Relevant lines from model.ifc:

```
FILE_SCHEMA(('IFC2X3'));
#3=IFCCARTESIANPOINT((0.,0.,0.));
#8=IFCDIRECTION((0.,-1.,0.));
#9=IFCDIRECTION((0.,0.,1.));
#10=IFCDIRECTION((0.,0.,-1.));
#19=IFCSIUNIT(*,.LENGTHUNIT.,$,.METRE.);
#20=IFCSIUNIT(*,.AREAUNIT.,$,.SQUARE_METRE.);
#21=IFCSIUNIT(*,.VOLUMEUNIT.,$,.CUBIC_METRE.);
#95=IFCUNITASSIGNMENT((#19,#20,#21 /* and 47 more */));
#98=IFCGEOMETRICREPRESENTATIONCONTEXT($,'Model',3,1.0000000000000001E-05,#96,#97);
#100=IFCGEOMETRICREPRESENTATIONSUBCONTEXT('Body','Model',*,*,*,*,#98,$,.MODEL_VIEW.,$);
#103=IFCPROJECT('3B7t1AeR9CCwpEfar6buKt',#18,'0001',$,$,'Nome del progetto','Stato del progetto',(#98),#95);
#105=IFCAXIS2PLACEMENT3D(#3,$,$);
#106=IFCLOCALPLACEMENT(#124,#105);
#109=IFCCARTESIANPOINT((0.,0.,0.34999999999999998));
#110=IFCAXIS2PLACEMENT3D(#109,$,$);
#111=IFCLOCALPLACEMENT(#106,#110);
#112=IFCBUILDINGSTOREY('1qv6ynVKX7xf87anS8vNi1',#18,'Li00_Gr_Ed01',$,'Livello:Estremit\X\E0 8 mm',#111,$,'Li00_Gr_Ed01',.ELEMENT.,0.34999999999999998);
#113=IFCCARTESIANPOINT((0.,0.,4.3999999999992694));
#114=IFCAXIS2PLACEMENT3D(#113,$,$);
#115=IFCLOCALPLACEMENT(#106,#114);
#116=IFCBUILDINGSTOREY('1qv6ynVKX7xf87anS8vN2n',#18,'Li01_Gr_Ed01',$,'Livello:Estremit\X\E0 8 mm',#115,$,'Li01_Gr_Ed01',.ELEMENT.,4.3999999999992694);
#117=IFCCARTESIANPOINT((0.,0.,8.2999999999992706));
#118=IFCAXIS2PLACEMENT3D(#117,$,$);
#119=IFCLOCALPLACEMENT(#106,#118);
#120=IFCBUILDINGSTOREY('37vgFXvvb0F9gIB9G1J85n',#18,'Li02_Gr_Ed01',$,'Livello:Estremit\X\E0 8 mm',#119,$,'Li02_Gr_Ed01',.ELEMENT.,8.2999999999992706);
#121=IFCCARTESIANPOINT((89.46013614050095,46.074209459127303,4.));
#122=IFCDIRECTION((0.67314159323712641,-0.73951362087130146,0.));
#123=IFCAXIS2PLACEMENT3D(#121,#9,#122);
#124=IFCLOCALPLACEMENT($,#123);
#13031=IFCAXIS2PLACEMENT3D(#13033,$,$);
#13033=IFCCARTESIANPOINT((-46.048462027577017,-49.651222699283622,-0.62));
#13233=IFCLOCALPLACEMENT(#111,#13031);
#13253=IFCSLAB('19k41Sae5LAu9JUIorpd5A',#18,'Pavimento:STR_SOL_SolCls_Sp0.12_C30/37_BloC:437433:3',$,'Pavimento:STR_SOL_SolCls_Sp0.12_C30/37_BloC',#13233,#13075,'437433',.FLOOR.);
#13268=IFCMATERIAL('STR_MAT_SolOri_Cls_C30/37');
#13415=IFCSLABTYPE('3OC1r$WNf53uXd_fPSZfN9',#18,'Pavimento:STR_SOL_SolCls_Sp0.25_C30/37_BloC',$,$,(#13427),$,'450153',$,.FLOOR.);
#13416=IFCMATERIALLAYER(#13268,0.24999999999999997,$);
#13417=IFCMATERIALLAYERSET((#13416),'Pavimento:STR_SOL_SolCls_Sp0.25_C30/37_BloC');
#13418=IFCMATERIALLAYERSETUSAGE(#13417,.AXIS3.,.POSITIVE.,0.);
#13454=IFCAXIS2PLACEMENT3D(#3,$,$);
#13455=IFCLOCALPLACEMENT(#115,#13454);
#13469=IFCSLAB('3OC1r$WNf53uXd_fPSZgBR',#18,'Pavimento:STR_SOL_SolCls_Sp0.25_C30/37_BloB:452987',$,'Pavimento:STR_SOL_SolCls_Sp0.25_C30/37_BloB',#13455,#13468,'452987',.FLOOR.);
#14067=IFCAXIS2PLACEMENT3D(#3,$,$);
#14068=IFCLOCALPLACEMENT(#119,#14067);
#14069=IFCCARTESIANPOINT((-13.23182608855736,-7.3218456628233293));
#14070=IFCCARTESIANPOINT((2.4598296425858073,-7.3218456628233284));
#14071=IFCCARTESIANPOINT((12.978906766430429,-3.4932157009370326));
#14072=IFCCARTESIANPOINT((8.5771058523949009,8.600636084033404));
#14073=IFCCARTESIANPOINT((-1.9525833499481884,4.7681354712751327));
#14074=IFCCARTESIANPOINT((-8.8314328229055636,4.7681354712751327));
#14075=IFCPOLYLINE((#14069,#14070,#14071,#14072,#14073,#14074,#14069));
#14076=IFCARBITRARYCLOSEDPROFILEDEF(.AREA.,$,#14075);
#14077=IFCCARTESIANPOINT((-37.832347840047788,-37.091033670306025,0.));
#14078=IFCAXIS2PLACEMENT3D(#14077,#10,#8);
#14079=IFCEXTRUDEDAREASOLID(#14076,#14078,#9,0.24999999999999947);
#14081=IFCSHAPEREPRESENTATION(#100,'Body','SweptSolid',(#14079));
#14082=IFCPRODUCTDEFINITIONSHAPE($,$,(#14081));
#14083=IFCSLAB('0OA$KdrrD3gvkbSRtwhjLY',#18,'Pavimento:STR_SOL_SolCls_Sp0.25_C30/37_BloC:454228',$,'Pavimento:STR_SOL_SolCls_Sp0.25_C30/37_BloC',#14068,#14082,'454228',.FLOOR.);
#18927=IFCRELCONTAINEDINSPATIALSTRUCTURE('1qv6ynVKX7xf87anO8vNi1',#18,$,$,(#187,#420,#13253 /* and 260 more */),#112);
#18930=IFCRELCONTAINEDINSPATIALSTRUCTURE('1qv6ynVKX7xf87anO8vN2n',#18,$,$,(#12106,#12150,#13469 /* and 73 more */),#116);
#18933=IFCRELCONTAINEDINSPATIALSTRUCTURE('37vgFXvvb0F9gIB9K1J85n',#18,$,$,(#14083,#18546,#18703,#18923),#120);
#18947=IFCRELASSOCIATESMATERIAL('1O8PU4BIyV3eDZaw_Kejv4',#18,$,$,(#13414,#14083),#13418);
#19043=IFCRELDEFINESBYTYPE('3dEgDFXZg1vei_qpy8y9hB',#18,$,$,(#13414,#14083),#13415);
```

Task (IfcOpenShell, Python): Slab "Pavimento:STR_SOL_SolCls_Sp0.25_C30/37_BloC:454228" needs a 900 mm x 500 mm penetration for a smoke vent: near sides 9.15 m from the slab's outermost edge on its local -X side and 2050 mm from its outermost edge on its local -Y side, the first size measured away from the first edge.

```python
import numpy as np
import ifcopenshell
import ifcopenshell.api.feature
import ifcopenshell.api.geometry
import ifcopenshell.api.root
import ifcopenshell.geom
import ifcopenshell.util.placement
import ifcopenshell.util.representation
import ifcopenshell.util.shape
import ifcopenshell.util.unit

model = ifcopenshell.open("model.ifc")
unit_scale = ifcopenshell.util.unit.calculate_unit_scale(model)
settings = ifcopenshell.geom.settings()


def volume(element):
    """Net volume in cubic metres, openings subtracted."""
    shape = ifcopenshell.geom.create_shape(settings, element)
    return ifcopenshell.util.shape.get_volume(shape.geometry)


slab = model.by_id(14083)
before = volume(slab)

# Extent in the slab's own axes, in metres. The edges named are its -X and -Y sides.
slab_shape = ifcopenshell.geom.create_shape(settings, slab)
vertices = ifcopenshell.util.shape.get_vertices(slab_shape.geometry)
x_min, y_min, bottom = vertices.min(axis=0)
top = vertices[:, 2].max()

opening = ifcopenshell.api.root.create_entity(model, ifc_class="IfcOpeningElement", name="Smoke vent opening")
context = ifcopenshell.util.representation.get_context(model, "Model", "Body", "MODEL_VIEW")
width, depth = 0.9, 0.5
outline = [(0.0, 0.0), (width, 0.0), (width, depth), (0.0, depth), (0.0, 0.0)]
# Overshoot both faces by 50 mm so the cut is clean.
shape = ifcopenshell.api.geometry.add_slab_representation(
    model, context=context, depth=top - bottom + 0.1, polyline=outline
)
ifcopenshell.api.geometry.assign_representation(model, product=opening, representation=shape)

matrix = ifcopenshell.util.placement.get_local_placement(slab.ObjectPlacement)
matrix[:, 3] = matrix @ np.append(np.array([x_min + 9.15, y_min + 2.05, bottom - 0.05]) / unit_scale, 1.0)
ifcopenshell.api.geometry.edit_object_placement(model, product=opening, matrix=matrix, is_si=False)
ifcopenshell.api.feature.add_feature(model, feature=opening, element=slab)

after = volume(slab)

print(f"slab volume {before:.3f} -> {after:.3f} m3")

model.write("model_edited.ifc")
```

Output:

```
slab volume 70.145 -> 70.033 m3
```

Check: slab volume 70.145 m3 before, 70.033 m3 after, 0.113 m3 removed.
